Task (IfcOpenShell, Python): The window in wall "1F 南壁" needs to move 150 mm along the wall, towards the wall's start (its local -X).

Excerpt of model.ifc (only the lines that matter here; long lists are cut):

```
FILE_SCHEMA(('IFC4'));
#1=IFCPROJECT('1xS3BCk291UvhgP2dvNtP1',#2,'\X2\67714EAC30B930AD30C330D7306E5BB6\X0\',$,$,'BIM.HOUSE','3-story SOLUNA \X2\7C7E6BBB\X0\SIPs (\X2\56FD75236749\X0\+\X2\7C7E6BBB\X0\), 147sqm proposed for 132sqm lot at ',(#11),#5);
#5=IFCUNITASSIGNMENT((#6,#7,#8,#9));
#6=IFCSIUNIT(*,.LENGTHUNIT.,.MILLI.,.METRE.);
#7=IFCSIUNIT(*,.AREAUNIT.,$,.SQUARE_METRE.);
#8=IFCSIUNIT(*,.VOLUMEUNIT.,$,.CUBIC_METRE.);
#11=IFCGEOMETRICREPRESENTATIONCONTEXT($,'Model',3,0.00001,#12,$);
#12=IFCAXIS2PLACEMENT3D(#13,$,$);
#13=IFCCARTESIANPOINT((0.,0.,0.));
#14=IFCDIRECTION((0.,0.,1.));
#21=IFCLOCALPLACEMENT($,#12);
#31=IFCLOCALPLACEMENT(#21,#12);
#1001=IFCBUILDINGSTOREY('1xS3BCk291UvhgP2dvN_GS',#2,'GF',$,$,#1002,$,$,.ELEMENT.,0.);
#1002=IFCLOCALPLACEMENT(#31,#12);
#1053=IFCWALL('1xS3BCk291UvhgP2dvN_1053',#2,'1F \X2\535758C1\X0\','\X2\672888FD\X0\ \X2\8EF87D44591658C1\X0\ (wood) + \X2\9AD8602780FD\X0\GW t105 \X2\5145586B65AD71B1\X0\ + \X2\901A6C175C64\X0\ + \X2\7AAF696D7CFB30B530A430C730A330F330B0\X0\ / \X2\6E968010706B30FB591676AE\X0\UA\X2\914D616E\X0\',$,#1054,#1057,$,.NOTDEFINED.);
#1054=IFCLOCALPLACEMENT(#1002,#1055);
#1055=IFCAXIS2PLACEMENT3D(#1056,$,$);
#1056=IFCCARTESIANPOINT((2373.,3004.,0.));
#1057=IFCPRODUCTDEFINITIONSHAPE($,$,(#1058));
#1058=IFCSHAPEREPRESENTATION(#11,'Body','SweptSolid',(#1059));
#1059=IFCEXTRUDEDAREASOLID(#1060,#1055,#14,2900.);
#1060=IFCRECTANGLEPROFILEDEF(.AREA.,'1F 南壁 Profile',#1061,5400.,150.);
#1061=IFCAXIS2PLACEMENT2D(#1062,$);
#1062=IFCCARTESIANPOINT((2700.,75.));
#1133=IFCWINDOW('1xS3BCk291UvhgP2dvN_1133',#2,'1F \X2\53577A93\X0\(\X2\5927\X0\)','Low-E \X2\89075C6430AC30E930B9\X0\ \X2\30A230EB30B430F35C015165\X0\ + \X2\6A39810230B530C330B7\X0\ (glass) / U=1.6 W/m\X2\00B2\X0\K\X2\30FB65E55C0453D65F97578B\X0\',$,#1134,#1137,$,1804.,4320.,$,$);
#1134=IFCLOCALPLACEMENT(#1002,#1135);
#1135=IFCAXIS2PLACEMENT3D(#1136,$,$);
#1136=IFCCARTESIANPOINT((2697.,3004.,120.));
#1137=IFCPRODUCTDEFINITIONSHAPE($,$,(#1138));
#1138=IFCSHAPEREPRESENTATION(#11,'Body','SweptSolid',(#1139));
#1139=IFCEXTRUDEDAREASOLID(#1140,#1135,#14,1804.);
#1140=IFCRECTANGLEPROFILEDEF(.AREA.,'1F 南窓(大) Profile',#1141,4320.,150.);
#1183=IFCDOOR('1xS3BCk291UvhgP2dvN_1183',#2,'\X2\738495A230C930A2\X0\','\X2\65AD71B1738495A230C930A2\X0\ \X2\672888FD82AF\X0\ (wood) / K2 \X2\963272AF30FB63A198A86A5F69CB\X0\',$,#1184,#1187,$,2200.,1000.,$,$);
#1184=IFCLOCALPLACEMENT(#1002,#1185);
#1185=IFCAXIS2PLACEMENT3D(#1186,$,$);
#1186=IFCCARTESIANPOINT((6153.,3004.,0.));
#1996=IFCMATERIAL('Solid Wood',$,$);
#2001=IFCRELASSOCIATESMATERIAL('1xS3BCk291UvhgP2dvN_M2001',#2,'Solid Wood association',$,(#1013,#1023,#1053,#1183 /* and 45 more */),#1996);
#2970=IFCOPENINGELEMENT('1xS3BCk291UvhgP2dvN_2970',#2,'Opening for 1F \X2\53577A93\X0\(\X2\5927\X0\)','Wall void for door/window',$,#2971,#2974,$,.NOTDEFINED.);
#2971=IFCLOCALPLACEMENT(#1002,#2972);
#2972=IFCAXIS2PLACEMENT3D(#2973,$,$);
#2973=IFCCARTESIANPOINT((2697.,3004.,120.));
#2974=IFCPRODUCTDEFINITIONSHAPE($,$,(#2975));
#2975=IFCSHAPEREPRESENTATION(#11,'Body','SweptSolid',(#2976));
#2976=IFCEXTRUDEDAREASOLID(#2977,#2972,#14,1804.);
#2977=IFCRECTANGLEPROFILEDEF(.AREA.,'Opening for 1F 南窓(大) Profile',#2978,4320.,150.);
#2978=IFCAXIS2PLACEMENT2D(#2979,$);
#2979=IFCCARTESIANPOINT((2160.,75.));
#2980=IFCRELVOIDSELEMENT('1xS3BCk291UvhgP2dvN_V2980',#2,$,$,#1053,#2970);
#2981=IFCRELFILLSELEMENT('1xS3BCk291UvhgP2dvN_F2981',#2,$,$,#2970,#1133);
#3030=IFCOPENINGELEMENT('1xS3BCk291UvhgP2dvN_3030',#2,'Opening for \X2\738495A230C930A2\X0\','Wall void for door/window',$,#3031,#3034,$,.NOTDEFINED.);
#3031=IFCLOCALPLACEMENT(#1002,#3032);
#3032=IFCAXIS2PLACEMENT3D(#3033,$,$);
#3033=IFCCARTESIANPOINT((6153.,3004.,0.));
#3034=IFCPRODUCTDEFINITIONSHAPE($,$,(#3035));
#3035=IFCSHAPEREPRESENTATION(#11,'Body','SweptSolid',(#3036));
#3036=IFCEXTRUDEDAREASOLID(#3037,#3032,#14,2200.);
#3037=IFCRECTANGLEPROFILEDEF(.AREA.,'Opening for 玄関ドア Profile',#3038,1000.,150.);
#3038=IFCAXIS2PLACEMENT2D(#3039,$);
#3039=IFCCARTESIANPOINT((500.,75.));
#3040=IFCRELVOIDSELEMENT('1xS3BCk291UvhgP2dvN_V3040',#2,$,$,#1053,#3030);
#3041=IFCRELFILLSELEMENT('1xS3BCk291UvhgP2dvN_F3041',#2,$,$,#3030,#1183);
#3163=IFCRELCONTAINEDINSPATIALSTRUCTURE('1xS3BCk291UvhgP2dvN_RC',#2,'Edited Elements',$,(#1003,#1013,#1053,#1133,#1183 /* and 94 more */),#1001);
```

```python
import ifcopenshell
import ifcopenshell.api.geometry
import ifcopenshell.util.placement
import ifcopenshell.util.unit

model = ifcopenshell.open("model.ifc")
unit_scale = ifcopenshell.util.unit.calculate_unit_scale(model)

window = model.by_id(1133)
opening = window.FillsVoids[0].RelatingOpeningElement
wall = opening.VoidsElements[0].RelatingBuildingElement

wall_matrix = ifcopenshell.util.placement.get_local_placement(wall.ObjectPlacement)
shift = wall_matrix[:3, 0] * -0.15 / unit_scale
before = ifcopenshell.util.placement.get_local_placement(window.ObjectPlacement)[:3, 3].copy()

# The window is not placed relative to its opening, so move both.
for product in (opening, window):
    matrix = ifcopenshell.util.placement.get_local_placement(product.ObjectPlacement)
    matrix[:3, 3] += shift
    ifcopenshell.api.geometry.edit_object_placement(model, product=product, matrix=matrix, is_si=False)

after = ifcopenshell.util.placement.get_local_placement(window.ObjectPlacement)[:3, 3]
print("window moved by", (after - before).round(3) + 0.0)

model.write("model_rev.ifc")
```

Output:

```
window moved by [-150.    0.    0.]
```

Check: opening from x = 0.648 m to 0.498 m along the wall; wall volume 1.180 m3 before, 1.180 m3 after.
